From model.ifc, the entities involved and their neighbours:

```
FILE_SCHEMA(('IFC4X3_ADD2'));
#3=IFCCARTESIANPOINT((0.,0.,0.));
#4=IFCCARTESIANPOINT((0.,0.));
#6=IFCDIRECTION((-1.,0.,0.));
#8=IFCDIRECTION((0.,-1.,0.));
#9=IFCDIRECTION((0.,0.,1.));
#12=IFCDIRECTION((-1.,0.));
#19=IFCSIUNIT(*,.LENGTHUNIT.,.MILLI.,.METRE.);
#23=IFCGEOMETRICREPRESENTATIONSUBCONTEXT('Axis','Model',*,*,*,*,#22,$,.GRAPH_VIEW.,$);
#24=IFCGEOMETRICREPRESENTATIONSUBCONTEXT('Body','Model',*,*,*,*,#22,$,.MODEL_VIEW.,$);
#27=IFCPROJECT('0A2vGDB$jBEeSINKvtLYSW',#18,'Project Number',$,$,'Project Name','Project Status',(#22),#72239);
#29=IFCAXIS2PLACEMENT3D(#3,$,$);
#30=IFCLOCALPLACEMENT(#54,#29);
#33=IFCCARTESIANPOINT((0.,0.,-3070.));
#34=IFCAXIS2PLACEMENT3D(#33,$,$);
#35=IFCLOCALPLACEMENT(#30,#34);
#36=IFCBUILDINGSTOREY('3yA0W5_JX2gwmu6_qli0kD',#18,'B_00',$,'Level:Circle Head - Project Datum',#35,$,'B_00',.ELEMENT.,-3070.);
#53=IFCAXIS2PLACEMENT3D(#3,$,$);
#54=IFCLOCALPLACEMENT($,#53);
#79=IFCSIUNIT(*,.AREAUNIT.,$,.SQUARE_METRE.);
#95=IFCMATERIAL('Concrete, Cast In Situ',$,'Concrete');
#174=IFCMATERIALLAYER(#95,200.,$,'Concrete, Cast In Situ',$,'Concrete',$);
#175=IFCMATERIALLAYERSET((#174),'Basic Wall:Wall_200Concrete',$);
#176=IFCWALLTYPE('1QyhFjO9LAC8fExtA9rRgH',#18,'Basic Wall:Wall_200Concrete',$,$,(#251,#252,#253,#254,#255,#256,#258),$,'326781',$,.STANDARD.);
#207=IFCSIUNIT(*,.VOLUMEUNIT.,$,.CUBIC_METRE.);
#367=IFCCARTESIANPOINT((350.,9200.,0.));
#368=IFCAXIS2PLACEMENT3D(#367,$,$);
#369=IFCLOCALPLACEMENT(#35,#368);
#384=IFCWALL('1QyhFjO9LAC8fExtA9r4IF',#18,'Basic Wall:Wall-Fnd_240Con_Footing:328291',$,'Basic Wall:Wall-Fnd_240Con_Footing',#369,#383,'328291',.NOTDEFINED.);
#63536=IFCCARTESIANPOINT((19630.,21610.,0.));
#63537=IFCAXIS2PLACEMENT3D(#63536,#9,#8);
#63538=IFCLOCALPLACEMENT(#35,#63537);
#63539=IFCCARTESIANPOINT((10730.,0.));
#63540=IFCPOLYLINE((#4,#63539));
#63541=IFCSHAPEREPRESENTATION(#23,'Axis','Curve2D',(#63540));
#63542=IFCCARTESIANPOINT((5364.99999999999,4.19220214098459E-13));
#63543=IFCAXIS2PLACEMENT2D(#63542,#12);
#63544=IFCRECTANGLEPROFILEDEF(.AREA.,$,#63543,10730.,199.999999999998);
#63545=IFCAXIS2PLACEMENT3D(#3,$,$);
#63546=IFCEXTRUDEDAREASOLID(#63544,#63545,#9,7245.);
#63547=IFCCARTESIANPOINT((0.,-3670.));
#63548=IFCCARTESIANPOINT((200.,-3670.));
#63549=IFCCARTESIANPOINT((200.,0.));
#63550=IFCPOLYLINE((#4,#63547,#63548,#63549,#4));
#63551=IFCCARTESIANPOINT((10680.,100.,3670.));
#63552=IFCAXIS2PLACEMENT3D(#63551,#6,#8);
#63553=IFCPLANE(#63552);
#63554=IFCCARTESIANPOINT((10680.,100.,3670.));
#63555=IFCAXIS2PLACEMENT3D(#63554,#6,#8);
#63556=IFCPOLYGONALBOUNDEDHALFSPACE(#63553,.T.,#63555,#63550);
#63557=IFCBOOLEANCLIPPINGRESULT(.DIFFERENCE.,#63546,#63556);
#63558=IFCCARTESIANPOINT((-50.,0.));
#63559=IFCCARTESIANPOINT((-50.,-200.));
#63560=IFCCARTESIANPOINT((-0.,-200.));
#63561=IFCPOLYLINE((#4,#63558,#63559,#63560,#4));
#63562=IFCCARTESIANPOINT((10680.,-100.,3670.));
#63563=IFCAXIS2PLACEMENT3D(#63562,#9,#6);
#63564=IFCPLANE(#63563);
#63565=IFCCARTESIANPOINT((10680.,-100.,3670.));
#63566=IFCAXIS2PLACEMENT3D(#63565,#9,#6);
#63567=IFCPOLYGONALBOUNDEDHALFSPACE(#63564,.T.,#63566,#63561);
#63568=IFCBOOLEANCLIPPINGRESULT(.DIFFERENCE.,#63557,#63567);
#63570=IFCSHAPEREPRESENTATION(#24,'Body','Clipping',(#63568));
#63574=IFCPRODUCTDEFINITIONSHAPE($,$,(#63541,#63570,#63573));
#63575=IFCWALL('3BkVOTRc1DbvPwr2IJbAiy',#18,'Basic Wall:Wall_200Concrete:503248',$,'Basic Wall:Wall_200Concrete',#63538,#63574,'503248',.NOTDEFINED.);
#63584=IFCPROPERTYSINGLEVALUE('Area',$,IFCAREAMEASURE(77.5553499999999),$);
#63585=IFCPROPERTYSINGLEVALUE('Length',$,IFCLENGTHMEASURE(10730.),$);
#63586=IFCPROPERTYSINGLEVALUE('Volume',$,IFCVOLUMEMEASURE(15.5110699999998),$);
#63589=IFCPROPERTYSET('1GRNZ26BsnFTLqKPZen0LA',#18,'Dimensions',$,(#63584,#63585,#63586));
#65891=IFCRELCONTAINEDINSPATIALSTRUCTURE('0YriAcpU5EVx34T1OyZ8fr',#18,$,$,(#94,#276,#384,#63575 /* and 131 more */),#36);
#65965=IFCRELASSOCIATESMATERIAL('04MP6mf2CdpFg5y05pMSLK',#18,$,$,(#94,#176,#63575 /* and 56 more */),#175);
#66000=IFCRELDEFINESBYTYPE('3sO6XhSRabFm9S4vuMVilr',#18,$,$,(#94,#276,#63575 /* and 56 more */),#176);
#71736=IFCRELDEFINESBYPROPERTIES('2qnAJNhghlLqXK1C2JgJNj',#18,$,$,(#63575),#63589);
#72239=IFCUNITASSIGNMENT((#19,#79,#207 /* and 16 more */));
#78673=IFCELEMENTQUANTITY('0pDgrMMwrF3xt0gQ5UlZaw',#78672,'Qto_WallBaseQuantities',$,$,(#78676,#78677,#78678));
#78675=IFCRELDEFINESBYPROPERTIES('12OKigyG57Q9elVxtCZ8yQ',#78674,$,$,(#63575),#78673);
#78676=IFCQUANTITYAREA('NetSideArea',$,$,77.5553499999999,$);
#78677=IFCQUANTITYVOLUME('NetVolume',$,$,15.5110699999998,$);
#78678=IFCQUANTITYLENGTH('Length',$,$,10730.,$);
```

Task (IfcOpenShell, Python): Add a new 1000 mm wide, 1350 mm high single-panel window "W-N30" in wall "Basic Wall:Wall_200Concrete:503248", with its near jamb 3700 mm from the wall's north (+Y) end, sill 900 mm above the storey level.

```python
import numpy as np
import ifcopenshell
import ifcopenshell.api.feature
import ifcopenshell.api.geometry
import ifcopenshell.api.pset
import ifcopenshell.api.root
import ifcopenshell.api.spatial
import ifcopenshell.geom
import ifcopenshell.util.element
import ifcopenshell.util.placement
import ifcopenshell.util.representation
import ifcopenshell.util.shape
import ifcopenshell.util.unit

model = ifcopenshell.open("model.ifc")
unit_scale = ifcopenshell.util.unit.calculate_unit_scale(model)
area_scale = ifcopenshell.util.unit.calculate_unit_scale(model, "AREAUNIT")
volume_scale = ifcopenshell.util.unit.calculate_unit_scale(model, "VOLUMEUNIT")
settings = ifcopenshell.geom.settings()


def volume(element):
    """Net volume in cubic metres, openings subtracted."""
    shape = ifcopenshell.geom.create_shape(settings, element)
    return ifcopenshell.util.shape.get_volume(shape.geometry)


wall = model.by_guid("3BkVOTRc1DbvPwr2IJbAiy")
storey = ifcopenshell.util.element.get_container(wall, ifc_class="IfcBuildingStorey")
context = ifcopenshell.util.representation.get_context(model, "Model", "Body", "MODEL_VIEW")
before = volume(wall)

width, height, from_end, sill = 1, 1.35, 3.7, 0.9  # metres

# The wall runs along its own X axis, and the end named is its -X end.
wall_shape = ifcopenshell.geom.create_shape(settings, wall)
x, y, z = ifcopenshell.util.shape.get_vertices(wall_shape.geometry).T
start = x.min() + from_end
face, thickness = float(y.min()), float(y.max() - y.min())
wall_matrix = ifcopenshell.util.placement.get_local_placement(wall.ObjectPlacement)
level = ifcopenshell.util.placement.get_local_placement(storey.ObjectPlacement)[2, 3]


def in_wall(x, y):
    """Placement at x, y metres in the wall's axes, at sill height."""
    matrix = wall_matrix.copy()
    matrix[:, 3] = wall_matrix @ np.array([x / unit_scale, y / unit_scale, 0.0, 1.0])
    matrix[2, 3] = level + sill / unit_scale
    return matrix


# Opening: a box that overshoots both wall faces by 50 mm.
opening = ifcopenshell.api.root.create_entity(model, ifc_class="IfcOpeningElement", predefined_type="OPENING")
box = ifcopenshell.api.geometry.add_wall_representation(
    model, context=context, length=width, height=height, thickness=thickness + 0.1
)
ifcopenshell.api.geometry.assign_representation(model, product=opening, representation=box)
ifcopenshell.api.geometry.edit_object_placement(model, product=opening, matrix=in_wall(start, face - 0.05), is_si=False)
ifcopenshell.api.feature.add_feature(model, feature=opening, element=wall)

window = ifcopenshell.api.root.create_entity(model, ifc_class="IfcWindow", name="W-N30", predefined_type="WINDOW")
window.OverallWidth, window.OverallHeight = width / unit_scale, height / unit_scale
window.PartitioningType = "SINGLE_PANEL"
body = ifcopenshell.api.geometry.add_window_representation(
    model,
    context=context,
    overall_width=window.OverallWidth,
    overall_height=window.OverallHeight,
    partition_type="SINGLE_PANEL",
)
ifcopenshell.api.geometry.assign_representation(model, product=window, representation=body)
ifcopenshell.api.spatial.assign_container(model, products=[window], relating_structure=storey)
ifcopenshell.api.feature.add_filling(model, opening=opening, element=window)

# Centre the window in the wall's thickness.
ifcopenshell.api.geometry.edit_object_placement(model, product=window, matrix=in_wall(start, face), is_si=False)
window_shape = ifcopenshell.geom.create_shape(settings, window)
depth = ifcopenshell.util.shape.get_vertices(window_shape.geometry)[:, 1]
offset = face + thickness / 2 - (depth.min() + depth.max()) / 2
ifcopenshell.api.geometry.edit_object_placement(model, product=window, matrix=in_wall(start, offset), is_si=False)

after = volume(wall)

# Update the wall's stored quantities.
pset = model.by_id(ifcopenshell.util.element.get_pset(wall, "Dimensions", should_inherit=False)["id"])
ifcopenshell.api.pset.edit_pset(model, pset=pset, properties={
    "Area": model.create_entity("IfcAreaMeasure", after / thickness / area_scale),
    "Volume": model.create_entity("IfcVolumeMeasure", after / volume_scale),
})
qto = model.by_id(ifcopenshell.util.element.get_pset(wall, "Qto_WallBaseQuantities", should_inherit=False)["id"])
ifcopenshell.api.pset.edit_qto(model, qto=qto, properties={
    "NetSideArea": after / thickness / area_scale,
    "NetVolume": after / volume_scale,
})

print(f"wall volume {before:.3f} -> {after:.3f} m3")

model.write("model_updated.ifc")
```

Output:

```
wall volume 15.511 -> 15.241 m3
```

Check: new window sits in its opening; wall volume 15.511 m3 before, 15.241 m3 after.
